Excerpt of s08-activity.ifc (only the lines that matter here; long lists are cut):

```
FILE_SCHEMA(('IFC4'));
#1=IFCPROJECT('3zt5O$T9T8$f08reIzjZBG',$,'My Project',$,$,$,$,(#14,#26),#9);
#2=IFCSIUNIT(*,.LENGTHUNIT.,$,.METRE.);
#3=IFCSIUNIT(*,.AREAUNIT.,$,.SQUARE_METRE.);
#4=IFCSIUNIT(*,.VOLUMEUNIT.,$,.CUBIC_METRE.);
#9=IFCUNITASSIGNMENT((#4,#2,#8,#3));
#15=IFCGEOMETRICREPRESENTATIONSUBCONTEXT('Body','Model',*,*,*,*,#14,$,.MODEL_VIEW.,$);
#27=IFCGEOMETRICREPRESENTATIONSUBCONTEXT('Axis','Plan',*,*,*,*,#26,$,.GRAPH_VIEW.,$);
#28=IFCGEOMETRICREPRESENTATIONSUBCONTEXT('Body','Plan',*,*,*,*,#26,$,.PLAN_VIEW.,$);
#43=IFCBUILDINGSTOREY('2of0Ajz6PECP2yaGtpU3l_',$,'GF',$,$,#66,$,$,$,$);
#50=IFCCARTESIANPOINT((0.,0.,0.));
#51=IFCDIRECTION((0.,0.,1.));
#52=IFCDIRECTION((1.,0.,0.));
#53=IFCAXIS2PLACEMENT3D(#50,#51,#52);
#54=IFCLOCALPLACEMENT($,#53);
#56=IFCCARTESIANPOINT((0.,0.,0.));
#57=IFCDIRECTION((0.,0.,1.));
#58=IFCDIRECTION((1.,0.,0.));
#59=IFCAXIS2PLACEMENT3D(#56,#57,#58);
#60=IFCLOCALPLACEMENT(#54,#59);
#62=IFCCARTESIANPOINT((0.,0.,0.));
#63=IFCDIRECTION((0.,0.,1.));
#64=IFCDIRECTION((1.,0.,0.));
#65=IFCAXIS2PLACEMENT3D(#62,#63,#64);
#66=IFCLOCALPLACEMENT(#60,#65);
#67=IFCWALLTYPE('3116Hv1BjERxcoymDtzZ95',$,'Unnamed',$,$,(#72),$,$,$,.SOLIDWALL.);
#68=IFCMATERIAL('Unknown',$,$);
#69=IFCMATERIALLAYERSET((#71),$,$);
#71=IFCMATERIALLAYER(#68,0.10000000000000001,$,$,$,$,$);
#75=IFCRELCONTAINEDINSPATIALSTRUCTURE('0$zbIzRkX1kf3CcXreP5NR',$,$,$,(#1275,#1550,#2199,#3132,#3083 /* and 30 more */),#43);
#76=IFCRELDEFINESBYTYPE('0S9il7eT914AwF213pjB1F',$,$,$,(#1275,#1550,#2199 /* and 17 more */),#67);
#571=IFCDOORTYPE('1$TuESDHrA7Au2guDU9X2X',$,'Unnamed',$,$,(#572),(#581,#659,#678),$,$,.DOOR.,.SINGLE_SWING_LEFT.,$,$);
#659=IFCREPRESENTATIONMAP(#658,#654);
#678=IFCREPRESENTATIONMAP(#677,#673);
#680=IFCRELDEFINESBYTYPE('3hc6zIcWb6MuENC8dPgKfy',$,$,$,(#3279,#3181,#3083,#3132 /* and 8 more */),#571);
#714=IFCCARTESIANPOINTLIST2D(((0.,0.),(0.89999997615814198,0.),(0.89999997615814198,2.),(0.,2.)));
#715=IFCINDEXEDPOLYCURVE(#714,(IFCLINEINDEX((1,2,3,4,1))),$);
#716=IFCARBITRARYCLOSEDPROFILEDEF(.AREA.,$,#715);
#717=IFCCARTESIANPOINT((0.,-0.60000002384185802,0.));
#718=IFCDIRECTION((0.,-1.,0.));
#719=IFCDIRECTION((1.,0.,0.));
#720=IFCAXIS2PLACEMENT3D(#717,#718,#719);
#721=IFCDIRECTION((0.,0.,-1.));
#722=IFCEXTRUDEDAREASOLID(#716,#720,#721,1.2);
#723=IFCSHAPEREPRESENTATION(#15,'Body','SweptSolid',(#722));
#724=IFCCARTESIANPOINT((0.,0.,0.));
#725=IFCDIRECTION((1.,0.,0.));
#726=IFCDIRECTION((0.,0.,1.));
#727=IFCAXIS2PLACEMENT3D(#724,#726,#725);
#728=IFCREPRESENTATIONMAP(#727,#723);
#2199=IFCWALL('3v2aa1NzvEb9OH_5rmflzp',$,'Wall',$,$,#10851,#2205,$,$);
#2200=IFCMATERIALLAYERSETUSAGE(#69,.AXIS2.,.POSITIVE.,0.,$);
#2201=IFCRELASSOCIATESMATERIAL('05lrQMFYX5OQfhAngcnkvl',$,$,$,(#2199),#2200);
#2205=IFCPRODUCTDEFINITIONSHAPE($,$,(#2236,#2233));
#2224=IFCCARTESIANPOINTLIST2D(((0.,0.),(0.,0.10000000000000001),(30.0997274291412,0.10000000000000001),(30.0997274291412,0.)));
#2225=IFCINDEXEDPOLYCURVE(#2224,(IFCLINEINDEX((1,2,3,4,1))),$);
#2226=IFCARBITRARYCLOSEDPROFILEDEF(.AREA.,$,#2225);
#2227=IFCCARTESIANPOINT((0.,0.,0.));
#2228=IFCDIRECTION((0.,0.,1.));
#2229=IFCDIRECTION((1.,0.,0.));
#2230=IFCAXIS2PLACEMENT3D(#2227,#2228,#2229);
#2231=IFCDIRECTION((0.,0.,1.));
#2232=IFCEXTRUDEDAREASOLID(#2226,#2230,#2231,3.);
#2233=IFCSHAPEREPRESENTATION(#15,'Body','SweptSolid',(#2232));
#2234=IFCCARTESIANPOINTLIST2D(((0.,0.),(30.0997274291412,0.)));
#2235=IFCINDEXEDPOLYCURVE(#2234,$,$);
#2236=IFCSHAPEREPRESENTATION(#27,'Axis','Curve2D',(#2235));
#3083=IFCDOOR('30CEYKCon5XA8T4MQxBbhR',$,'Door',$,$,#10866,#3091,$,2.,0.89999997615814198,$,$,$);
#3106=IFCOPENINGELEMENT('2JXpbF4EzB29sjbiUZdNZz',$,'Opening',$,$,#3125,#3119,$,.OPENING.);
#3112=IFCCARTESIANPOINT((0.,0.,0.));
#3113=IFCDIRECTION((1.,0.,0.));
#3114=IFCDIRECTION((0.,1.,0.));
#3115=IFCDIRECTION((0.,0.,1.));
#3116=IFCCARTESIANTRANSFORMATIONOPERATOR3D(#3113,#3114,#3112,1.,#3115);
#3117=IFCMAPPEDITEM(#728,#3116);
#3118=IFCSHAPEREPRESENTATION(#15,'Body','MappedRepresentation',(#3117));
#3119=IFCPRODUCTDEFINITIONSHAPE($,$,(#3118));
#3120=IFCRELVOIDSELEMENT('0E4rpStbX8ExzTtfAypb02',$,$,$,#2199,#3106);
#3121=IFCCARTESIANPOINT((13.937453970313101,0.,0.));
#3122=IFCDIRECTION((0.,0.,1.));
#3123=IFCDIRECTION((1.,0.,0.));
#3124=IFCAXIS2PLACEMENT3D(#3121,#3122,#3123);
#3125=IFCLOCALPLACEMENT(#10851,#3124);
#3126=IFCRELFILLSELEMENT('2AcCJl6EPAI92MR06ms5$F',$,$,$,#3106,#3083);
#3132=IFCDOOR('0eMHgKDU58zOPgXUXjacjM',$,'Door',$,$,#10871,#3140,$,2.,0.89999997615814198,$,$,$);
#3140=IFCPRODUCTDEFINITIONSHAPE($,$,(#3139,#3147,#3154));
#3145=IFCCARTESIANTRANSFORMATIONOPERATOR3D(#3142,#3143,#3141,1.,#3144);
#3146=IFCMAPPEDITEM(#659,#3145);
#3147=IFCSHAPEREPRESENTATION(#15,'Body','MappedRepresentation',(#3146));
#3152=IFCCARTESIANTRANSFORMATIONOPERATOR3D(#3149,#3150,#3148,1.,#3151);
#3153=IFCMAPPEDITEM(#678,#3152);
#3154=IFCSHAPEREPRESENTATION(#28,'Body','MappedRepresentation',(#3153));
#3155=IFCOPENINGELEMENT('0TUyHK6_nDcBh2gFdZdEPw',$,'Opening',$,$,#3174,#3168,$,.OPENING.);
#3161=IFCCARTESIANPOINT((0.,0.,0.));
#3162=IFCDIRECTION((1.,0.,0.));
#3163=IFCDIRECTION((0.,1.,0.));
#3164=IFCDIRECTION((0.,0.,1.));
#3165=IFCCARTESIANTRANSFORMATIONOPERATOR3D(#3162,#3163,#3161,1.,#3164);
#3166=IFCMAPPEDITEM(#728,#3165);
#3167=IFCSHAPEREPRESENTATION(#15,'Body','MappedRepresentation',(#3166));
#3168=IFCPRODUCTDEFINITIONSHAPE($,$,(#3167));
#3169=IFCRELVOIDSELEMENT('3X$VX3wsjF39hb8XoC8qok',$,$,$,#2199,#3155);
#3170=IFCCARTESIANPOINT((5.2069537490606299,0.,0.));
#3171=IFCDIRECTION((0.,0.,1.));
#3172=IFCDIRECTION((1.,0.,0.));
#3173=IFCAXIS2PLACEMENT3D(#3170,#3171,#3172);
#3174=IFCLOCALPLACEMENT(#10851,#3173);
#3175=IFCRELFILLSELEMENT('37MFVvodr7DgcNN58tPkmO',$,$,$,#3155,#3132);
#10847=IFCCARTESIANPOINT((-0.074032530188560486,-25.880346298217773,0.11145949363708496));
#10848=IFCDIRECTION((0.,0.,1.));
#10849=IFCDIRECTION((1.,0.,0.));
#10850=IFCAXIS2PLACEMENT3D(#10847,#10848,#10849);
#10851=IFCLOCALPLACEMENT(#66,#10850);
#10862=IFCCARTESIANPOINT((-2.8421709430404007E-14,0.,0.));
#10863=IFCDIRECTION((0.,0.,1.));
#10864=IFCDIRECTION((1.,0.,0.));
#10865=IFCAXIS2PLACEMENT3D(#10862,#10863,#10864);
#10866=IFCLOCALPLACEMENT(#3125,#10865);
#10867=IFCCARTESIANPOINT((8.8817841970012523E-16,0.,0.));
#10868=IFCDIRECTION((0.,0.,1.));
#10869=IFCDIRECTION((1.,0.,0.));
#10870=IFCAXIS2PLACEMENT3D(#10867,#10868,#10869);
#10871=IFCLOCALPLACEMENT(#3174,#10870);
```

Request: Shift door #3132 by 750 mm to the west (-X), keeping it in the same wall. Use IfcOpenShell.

```python
import ifcopenshell
import ifcopenshell.api.geometry
import ifcopenshell.util.placement

model = ifcopenshell.open("s08-activity.ifc")

door = model.by_id(3132)
opening = door.FillsVoids[0].RelatingOpeningElement
wall = opening.VoidsElements[0].RelatingBuildingElement

wall_matrix = ifcopenshell.util.placement.get_local_placement(wall.ObjectPlacement)
shift = wall_matrix[:3, 0] * -0.75
before = ifcopenshell.util.placement.get_local_placement(door.ObjectPlacement)[:3, 3].copy()

# The door is placed relative to its opening, so it follows when the opening moves.
matrix = ifcopenshell.util.placement.get_local_placement(opening.ObjectPlacement)
matrix[:3, 3] += shift
ifcopenshell.api.geometry.edit_object_placement(
    model, product=opening, matrix=matrix, is_si=False, should_transform_children=True
)

after = ifcopenshell.util.placement.get_local_placement(door.ObjectPlacement)[:3, 3]
print("door moved by", (after - before).round(3) + 0.0)

model.write("s08-activity_rev.ifc")
```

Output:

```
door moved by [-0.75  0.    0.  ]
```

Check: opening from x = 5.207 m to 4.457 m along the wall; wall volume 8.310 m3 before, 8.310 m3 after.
